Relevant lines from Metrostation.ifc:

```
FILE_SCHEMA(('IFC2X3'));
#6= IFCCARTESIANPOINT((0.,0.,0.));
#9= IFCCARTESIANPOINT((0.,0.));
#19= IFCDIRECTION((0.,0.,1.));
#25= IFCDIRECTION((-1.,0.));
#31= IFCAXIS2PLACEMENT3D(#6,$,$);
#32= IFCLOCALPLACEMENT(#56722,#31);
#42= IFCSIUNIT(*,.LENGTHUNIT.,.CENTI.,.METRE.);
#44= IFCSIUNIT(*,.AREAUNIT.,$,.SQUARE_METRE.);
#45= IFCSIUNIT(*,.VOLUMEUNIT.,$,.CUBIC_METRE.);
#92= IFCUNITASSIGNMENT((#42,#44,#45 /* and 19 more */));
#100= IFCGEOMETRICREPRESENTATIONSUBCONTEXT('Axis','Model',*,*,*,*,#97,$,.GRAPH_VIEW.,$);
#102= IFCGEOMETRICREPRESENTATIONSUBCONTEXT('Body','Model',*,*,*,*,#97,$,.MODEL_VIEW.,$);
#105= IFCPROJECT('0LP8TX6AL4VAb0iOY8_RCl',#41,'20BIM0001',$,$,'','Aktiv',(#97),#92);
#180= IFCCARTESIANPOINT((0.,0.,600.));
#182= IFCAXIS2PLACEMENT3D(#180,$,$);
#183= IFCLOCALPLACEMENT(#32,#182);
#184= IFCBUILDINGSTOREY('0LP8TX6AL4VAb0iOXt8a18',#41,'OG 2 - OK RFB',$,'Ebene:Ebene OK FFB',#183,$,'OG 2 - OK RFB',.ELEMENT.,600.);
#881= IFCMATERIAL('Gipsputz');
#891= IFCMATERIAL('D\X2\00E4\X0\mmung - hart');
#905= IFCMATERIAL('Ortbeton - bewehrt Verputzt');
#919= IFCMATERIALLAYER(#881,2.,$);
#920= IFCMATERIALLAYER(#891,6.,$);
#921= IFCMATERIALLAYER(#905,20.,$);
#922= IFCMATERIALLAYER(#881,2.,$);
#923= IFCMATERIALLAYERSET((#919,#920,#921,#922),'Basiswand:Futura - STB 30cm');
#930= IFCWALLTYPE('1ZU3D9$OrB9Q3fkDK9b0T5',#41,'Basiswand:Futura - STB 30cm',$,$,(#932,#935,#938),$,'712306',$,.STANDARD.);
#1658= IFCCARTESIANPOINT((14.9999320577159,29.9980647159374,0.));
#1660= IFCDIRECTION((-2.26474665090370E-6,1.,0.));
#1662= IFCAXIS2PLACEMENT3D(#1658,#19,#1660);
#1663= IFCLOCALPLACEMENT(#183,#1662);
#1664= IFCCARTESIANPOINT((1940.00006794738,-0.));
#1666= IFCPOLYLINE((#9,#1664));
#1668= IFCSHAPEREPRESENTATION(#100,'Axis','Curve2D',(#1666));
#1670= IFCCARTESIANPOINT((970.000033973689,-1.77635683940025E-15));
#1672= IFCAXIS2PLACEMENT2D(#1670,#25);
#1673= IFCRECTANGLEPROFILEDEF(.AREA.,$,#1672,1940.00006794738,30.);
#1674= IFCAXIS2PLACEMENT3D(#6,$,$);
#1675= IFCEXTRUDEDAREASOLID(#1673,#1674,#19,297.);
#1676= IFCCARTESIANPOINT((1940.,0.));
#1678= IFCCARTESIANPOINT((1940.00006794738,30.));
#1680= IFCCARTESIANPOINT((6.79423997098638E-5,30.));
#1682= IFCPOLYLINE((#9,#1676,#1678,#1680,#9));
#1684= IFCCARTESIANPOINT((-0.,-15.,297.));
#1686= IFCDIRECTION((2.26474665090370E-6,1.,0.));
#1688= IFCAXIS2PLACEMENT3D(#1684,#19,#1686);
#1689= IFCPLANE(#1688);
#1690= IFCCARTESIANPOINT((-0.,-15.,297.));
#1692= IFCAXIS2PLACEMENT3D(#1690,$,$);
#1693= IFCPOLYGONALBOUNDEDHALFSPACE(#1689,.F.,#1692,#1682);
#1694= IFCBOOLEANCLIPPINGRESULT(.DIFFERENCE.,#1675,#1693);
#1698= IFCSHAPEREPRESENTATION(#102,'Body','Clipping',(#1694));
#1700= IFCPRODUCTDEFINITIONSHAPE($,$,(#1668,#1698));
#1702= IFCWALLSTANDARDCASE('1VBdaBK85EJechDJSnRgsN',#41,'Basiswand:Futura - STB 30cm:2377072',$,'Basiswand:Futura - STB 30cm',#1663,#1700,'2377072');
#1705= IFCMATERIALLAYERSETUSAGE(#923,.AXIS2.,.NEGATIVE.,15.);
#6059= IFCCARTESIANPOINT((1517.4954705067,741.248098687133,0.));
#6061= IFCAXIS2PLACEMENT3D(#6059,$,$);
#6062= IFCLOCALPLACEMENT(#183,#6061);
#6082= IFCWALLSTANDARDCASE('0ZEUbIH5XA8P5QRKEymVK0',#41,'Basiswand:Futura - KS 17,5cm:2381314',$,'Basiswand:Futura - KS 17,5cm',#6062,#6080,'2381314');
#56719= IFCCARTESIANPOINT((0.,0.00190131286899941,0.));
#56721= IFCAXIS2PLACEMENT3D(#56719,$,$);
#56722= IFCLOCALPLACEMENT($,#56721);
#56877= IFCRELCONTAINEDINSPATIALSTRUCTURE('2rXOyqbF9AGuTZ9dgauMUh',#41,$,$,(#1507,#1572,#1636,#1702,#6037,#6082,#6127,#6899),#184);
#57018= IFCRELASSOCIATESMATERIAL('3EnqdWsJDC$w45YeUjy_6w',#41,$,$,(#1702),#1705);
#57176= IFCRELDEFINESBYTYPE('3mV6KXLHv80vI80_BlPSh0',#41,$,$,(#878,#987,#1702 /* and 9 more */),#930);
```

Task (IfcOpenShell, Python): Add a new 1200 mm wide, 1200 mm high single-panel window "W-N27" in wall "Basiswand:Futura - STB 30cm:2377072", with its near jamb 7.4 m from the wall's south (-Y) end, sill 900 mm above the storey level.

```python
import numpy as np
import ifcopenshell
import ifcopenshell.api.feature
import ifcopenshell.api.geometry
import ifcopenshell.api.root
import ifcopenshell.api.spatial
import ifcopenshell.api.type
import ifcopenshell.geom
import ifcopenshell.util.element
import ifcopenshell.util.placement
import ifcopenshell.util.representation
import ifcopenshell.util.shape
import ifcopenshell.util.unit

model = ifcopenshell.open("Metrostation.ifc")
unit_scale = ifcopenshell.util.unit.calculate_unit_scale(model)
settings = ifcopenshell.geom.settings()


def volume(element):
    """Net volume in cubic metres, openings subtracted."""
    shape = ifcopenshell.geom.create_shape(settings, element)
    return ifcopenshell.util.shape.get_volume(shape.geometry)


wall = model.by_id(1702)
storey = ifcopenshell.util.element.get_container(wall, ifc_class="IfcBuildingStorey")
context = ifcopenshell.util.representation.get_context(model, "Model", "Body", "MODEL_VIEW")
before = volume(wall)

width, height, from_end, sill = 1.2, 1.2, 7.4, 0.9  # metres

# The wall runs along its own X axis, and the end named is its -X end.
wall_shape = ifcopenshell.geom.create_shape(settings, wall)
x, y, z = ifcopenshell.util.shape.get_vertices(wall_shape.geometry).T
start = x.min() + from_end
face, thickness = float(y.min()), float(y.max() - y.min())
wall_matrix = ifcopenshell.util.placement.get_local_placement(wall.ObjectPlacement)
level = ifcopenshell.util.placement.get_local_placement(storey.ObjectPlacement)[2, 3]


def in_wall(x, y):
    """Placement at x, y metres in the wall's axes, at sill height."""
    matrix = wall_matrix.copy()
    matrix[:, 3] = wall_matrix @ np.array([x / unit_scale, y / unit_scale, 0.0, 1.0])
    matrix[2, 3] = level + sill / unit_scale
    return matrix


# Opening: a box that overshoots both wall faces by 50 mm.
opening = ifcopenshell.api.root.create_entity(model, ifc_class="IfcOpeningElement")
box = ifcopenshell.api.geometry.add_wall_representation(
    model, context=context, length=width, height=height, thickness=thickness + 0.1
)
ifcopenshell.api.geometry.assign_representation(model, product=opening, representation=box)
ifcopenshell.api.geometry.edit_object_placement(model, product=opening, matrix=in_wall(start, face - 0.05), is_si=False)
ifcopenshell.api.feature.add_feature(model, feature=opening, element=wall)

window = ifcopenshell.api.root.create_entity(model, ifc_class="IfcWindow", name="W-N27")
window.OverallWidth, window.OverallHeight = width / unit_scale, height / unit_scale
body = ifcopenshell.api.geometry.add_window_representation(
    model,
    context=context,
    overall_width=window.OverallWidth,
    overall_height=window.OverallHeight,
    partition_type="SINGLE_PANEL",
)
ifcopenshell.api.geometry.assign_representation(model, product=window, representation=body)
ifcopenshell.api.spatial.assign_container(model, products=[window], relating_structure=storey)
fills = ifcopenshell.api.feature.add_filling(model, opening=opening, element=window)
fills.OwnerHistory = window.OwnerHistory  # required in IFC2X3

# IFC2X3 keeps the operation on the window style.
style = ifcopenshell.api.root.create_entity(model, ifc_class="IfcWindowStyle", name="W-N27")
style.OperationType, style.ConstructionType = "SINGLE_PANEL", "NOTDEFINED"
style.ParameterTakesPrecedence = style.Sizeable = False
ifcopenshell.api.type.assign_type(model, related_objects=[window], relating_type=style)

# Centre the window in the wall's thickness.
ifcopenshell.api.geometry.edit_object_placement(model, product=window, matrix=in_wall(start, face), is_si=False)
window_shape = ifcopenshell.geom.create_shape(settings, window)
depth = ifcopenshell.util.shape.get_vertices(window_shape.geometry)[:, 1]
offset = face + thickness / 2 - (depth.min() + depth.max()) / 2
ifcopenshell.api.geometry.edit_object_placement(model, product=window, matrix=in_wall(start, offset), is_si=False)

after = volume(wall)

print(f"wall volume {before:.3f} -> {after:.3f} m3")

model.write("Metrostation-out.ifc")
```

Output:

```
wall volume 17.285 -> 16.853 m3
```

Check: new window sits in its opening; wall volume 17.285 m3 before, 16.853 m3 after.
